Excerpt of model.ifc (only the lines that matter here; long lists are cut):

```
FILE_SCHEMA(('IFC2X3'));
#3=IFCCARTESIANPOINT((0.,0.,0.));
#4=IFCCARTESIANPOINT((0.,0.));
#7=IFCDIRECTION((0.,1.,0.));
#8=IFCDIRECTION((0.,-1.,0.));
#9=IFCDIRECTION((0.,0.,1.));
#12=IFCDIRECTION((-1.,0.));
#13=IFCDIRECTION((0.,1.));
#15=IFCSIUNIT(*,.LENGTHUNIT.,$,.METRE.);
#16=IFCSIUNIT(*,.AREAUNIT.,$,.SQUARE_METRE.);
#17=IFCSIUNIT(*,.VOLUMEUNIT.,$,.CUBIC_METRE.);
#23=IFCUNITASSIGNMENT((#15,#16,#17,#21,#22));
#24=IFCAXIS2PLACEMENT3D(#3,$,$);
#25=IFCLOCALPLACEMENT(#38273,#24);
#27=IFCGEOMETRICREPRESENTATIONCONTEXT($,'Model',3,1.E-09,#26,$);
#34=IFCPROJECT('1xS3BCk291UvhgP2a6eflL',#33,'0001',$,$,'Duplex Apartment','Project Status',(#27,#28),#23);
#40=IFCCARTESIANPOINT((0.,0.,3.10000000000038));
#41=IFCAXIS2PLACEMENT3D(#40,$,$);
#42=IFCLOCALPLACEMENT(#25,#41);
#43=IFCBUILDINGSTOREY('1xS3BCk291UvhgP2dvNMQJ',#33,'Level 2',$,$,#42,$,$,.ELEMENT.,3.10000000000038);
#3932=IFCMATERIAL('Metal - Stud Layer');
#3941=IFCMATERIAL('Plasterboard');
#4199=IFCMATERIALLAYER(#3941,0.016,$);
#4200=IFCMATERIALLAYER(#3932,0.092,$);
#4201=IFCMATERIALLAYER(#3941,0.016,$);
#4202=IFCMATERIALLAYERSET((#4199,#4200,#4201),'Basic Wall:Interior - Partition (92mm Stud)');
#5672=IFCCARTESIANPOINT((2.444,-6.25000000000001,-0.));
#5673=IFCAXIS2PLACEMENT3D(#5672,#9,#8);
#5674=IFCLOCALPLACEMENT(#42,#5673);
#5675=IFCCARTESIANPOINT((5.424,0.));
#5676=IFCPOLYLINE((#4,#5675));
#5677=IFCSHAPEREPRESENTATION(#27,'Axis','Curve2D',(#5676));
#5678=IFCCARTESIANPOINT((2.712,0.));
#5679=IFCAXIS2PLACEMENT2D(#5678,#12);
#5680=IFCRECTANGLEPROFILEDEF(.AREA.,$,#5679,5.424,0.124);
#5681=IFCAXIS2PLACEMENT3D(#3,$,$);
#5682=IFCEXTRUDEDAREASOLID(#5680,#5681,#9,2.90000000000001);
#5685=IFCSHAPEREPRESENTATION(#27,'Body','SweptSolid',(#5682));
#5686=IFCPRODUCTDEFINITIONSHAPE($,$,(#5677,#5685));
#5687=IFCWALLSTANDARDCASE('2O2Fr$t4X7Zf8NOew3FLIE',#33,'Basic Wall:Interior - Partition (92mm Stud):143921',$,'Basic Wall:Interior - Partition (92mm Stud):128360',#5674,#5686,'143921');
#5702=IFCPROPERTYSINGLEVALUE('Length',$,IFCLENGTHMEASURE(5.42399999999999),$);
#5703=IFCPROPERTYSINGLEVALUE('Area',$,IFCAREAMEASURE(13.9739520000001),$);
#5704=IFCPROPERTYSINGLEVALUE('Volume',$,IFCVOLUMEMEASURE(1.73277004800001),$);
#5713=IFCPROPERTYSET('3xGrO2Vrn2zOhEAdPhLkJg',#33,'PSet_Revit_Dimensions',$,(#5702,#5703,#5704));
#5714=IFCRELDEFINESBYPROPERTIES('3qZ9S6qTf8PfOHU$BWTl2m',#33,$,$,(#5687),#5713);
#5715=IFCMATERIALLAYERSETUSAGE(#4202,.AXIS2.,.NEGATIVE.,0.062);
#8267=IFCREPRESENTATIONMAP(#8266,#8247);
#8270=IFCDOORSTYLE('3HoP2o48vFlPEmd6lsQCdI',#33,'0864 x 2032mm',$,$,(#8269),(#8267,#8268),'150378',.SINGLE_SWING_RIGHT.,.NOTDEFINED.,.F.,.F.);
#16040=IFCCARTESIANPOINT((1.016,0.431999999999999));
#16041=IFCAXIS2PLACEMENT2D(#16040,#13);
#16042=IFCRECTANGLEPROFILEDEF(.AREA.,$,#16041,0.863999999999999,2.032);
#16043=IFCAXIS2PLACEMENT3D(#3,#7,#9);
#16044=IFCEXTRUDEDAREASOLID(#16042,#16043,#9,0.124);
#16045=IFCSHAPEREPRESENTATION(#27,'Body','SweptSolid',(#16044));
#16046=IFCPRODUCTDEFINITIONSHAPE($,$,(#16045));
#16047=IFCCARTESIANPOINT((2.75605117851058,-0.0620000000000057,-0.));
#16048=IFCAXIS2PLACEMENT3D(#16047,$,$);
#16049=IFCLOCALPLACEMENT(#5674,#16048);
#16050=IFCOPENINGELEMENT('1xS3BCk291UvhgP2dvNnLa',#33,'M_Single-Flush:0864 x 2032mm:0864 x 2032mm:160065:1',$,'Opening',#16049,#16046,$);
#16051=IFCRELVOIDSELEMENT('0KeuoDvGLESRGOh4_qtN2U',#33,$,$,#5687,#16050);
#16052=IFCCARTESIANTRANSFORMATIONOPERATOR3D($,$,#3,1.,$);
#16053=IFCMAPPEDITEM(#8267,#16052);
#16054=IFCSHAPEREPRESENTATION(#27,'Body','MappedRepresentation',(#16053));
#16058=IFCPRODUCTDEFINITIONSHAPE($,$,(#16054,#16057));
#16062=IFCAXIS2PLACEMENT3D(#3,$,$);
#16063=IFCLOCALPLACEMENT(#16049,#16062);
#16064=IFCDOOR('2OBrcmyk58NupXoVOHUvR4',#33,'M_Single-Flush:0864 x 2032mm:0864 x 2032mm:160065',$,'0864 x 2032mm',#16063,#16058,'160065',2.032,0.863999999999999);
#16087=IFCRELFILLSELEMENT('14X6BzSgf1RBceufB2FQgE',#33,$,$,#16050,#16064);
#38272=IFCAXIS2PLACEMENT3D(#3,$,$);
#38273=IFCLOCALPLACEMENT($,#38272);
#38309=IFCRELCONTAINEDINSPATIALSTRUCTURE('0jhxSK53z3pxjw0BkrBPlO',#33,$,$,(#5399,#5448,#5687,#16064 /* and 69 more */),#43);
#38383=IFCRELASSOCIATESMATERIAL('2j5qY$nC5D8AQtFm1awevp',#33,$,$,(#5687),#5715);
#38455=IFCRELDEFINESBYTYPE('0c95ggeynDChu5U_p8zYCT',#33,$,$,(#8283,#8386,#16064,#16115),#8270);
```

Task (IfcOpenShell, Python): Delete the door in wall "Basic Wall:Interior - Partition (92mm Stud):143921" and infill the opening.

```python
import ifcopenshell
import ifcopenshell.api.feature
import ifcopenshell.api.pset
import ifcopenshell.api.root
import ifcopenshell.geom
import ifcopenshell.util.element
import ifcopenshell.util.shape
import ifcopenshell.util.unit

model = ifcopenshell.open("model.ifc")
area_scale = ifcopenshell.util.unit.calculate_unit_scale(model, "AREAUNIT")
volume_scale = ifcopenshell.util.unit.calculate_unit_scale(model, "VOLUMEUNIT")
settings = ifcopenshell.geom.settings()


def volume(element):
    """Net volume in cubic metres, openings subtracted."""
    shape = ifcopenshell.geom.create_shape(settings, element)
    return ifcopenshell.util.shape.get_volume(shape.geometry)


door = model.by_guid("2OBrcmyk58NupXoVOHUvR4")
opening = door.FillsVoids[0].RelatingOpeningElement
wall = opening.VoidsElements[0].RelatingBuildingElement
before = volume(wall)

ifcopenshell.api.root.remove_product(model, product=door)
ifcopenshell.api.feature.remove_feature(model, feature=opening)

after = volume(wall)
thickness = 0.124  # wall thickness in metres

# Update the wall's stored quantities.
pset = model.by_id(ifcopenshell.util.element.get_pset(wall, "PSet_Revit_Dimensions", should_inherit=False)["id"])
ifcopenshell.api.pset.edit_pset(model, pset=pset, properties={
    "Area": model.create_entity("IfcAreaMeasure", after / thickness / area_scale),
    "Volume": model.create_entity("IfcVolumeMeasure", after / volume_scale),
})

print(f"wall volume {before:.3f} -> {after:.3f} m3")

model.write("model_edited.ifc")
```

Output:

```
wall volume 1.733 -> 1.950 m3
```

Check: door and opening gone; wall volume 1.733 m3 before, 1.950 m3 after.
